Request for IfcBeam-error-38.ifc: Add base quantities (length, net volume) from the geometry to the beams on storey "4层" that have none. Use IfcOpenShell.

First a look at what the model holds.

```python
import ifcopenshell
import ifcopenshell.util.element
import ifcopenshell.util.unit

model = ifcopenshell.open("IfcBeam-error-38.ifc")
print(model.schema)
for unit_type in ("LENGTHUNIT", "AREAUNIT", "VOLUMEUNIT"):
    print(unit_type, ifcopenshell.util.unit.calculate_unit_scale(model, unit_type))
storey = next(s for s in model.by_type("IfcBuildingStorey") if s.Name == "4层")
beams = [e for e in ifcopenshell.util.element.get_decomposition(storey) if e.is_a("IfcBeam")]
for e in sorted(beams, key=lambda e: e.id()):
    print(e.id(), e.is_a(), e.Name, list(ifcopenshell.util.element.get_psets(e, qtos_only=True)), sep=" | ")
```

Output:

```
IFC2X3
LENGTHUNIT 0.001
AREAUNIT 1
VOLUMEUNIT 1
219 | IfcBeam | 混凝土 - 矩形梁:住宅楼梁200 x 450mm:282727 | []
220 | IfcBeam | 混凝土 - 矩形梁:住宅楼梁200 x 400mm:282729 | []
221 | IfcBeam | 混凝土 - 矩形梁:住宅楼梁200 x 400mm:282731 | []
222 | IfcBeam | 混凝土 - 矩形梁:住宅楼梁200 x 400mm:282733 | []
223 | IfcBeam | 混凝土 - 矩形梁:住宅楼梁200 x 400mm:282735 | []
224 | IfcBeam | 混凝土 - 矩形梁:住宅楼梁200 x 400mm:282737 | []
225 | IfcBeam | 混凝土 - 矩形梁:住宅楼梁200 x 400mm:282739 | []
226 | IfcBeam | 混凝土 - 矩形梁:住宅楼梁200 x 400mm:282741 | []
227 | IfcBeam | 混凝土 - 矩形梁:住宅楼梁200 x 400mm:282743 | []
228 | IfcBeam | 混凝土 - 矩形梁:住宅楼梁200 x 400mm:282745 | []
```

```python
import ifcopenshell
import ifcopenshell.api.pset
import ifcopenshell.geom
import ifcopenshell.util.element
import ifcopenshell.util.shape
import ifcopenshell.util.unit

model = ifcopenshell.open("IfcBeam-error-38.ifc")
unit_scale = ifcopenshell.util.unit.calculate_unit_scale(model)
volume_scale = ifcopenshell.util.unit.calculate_unit_scale(model, "VOLUMEUNIT")
settings = ifcopenshell.geom.settings()

storey = next(s for s in model.by_type("IfcBuildingStorey") if s.Name == "4层")
beams = [e for e in ifcopenshell.util.element.get_decomposition(storey) if e.is_a("IfcBeam")]

for e in sorted(beams, key=lambda e: e.id()):
    if ifcopenshell.util.element.get_psets(e, qtos_only=True, should_inherit=False):
        continue
    # Geometry comes back in metres, in the element's own axes.
    shape = ifcopenshell.geom.create_shape(settings, e)
    values = {
        "Length": ifcopenshell.util.shape.get_max_xyz(shape.geometry) / unit_scale,
        "NetVolume": ifcopenshell.util.shape.get_volume(shape.geometry) / volume_scale,
    }
    qto = ifcopenshell.api.pset.add_qto(model, product=e, name="BaseQuantities")
    ifcopenshell.api.pset.edit_qto(model, qto=qto, properties=values)
    print(e.id(), {k: round(v, 3) for k, v in values.items()})

model.write("IfcBeam-error-38_edited.ifc")
```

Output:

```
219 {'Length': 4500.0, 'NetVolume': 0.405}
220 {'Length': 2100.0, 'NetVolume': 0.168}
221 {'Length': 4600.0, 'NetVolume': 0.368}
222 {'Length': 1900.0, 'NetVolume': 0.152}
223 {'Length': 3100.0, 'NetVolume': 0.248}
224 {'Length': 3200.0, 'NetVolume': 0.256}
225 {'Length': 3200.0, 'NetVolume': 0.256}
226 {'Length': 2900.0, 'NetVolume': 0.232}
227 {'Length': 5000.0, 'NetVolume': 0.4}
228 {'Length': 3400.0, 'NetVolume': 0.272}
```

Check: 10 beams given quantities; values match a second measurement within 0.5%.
